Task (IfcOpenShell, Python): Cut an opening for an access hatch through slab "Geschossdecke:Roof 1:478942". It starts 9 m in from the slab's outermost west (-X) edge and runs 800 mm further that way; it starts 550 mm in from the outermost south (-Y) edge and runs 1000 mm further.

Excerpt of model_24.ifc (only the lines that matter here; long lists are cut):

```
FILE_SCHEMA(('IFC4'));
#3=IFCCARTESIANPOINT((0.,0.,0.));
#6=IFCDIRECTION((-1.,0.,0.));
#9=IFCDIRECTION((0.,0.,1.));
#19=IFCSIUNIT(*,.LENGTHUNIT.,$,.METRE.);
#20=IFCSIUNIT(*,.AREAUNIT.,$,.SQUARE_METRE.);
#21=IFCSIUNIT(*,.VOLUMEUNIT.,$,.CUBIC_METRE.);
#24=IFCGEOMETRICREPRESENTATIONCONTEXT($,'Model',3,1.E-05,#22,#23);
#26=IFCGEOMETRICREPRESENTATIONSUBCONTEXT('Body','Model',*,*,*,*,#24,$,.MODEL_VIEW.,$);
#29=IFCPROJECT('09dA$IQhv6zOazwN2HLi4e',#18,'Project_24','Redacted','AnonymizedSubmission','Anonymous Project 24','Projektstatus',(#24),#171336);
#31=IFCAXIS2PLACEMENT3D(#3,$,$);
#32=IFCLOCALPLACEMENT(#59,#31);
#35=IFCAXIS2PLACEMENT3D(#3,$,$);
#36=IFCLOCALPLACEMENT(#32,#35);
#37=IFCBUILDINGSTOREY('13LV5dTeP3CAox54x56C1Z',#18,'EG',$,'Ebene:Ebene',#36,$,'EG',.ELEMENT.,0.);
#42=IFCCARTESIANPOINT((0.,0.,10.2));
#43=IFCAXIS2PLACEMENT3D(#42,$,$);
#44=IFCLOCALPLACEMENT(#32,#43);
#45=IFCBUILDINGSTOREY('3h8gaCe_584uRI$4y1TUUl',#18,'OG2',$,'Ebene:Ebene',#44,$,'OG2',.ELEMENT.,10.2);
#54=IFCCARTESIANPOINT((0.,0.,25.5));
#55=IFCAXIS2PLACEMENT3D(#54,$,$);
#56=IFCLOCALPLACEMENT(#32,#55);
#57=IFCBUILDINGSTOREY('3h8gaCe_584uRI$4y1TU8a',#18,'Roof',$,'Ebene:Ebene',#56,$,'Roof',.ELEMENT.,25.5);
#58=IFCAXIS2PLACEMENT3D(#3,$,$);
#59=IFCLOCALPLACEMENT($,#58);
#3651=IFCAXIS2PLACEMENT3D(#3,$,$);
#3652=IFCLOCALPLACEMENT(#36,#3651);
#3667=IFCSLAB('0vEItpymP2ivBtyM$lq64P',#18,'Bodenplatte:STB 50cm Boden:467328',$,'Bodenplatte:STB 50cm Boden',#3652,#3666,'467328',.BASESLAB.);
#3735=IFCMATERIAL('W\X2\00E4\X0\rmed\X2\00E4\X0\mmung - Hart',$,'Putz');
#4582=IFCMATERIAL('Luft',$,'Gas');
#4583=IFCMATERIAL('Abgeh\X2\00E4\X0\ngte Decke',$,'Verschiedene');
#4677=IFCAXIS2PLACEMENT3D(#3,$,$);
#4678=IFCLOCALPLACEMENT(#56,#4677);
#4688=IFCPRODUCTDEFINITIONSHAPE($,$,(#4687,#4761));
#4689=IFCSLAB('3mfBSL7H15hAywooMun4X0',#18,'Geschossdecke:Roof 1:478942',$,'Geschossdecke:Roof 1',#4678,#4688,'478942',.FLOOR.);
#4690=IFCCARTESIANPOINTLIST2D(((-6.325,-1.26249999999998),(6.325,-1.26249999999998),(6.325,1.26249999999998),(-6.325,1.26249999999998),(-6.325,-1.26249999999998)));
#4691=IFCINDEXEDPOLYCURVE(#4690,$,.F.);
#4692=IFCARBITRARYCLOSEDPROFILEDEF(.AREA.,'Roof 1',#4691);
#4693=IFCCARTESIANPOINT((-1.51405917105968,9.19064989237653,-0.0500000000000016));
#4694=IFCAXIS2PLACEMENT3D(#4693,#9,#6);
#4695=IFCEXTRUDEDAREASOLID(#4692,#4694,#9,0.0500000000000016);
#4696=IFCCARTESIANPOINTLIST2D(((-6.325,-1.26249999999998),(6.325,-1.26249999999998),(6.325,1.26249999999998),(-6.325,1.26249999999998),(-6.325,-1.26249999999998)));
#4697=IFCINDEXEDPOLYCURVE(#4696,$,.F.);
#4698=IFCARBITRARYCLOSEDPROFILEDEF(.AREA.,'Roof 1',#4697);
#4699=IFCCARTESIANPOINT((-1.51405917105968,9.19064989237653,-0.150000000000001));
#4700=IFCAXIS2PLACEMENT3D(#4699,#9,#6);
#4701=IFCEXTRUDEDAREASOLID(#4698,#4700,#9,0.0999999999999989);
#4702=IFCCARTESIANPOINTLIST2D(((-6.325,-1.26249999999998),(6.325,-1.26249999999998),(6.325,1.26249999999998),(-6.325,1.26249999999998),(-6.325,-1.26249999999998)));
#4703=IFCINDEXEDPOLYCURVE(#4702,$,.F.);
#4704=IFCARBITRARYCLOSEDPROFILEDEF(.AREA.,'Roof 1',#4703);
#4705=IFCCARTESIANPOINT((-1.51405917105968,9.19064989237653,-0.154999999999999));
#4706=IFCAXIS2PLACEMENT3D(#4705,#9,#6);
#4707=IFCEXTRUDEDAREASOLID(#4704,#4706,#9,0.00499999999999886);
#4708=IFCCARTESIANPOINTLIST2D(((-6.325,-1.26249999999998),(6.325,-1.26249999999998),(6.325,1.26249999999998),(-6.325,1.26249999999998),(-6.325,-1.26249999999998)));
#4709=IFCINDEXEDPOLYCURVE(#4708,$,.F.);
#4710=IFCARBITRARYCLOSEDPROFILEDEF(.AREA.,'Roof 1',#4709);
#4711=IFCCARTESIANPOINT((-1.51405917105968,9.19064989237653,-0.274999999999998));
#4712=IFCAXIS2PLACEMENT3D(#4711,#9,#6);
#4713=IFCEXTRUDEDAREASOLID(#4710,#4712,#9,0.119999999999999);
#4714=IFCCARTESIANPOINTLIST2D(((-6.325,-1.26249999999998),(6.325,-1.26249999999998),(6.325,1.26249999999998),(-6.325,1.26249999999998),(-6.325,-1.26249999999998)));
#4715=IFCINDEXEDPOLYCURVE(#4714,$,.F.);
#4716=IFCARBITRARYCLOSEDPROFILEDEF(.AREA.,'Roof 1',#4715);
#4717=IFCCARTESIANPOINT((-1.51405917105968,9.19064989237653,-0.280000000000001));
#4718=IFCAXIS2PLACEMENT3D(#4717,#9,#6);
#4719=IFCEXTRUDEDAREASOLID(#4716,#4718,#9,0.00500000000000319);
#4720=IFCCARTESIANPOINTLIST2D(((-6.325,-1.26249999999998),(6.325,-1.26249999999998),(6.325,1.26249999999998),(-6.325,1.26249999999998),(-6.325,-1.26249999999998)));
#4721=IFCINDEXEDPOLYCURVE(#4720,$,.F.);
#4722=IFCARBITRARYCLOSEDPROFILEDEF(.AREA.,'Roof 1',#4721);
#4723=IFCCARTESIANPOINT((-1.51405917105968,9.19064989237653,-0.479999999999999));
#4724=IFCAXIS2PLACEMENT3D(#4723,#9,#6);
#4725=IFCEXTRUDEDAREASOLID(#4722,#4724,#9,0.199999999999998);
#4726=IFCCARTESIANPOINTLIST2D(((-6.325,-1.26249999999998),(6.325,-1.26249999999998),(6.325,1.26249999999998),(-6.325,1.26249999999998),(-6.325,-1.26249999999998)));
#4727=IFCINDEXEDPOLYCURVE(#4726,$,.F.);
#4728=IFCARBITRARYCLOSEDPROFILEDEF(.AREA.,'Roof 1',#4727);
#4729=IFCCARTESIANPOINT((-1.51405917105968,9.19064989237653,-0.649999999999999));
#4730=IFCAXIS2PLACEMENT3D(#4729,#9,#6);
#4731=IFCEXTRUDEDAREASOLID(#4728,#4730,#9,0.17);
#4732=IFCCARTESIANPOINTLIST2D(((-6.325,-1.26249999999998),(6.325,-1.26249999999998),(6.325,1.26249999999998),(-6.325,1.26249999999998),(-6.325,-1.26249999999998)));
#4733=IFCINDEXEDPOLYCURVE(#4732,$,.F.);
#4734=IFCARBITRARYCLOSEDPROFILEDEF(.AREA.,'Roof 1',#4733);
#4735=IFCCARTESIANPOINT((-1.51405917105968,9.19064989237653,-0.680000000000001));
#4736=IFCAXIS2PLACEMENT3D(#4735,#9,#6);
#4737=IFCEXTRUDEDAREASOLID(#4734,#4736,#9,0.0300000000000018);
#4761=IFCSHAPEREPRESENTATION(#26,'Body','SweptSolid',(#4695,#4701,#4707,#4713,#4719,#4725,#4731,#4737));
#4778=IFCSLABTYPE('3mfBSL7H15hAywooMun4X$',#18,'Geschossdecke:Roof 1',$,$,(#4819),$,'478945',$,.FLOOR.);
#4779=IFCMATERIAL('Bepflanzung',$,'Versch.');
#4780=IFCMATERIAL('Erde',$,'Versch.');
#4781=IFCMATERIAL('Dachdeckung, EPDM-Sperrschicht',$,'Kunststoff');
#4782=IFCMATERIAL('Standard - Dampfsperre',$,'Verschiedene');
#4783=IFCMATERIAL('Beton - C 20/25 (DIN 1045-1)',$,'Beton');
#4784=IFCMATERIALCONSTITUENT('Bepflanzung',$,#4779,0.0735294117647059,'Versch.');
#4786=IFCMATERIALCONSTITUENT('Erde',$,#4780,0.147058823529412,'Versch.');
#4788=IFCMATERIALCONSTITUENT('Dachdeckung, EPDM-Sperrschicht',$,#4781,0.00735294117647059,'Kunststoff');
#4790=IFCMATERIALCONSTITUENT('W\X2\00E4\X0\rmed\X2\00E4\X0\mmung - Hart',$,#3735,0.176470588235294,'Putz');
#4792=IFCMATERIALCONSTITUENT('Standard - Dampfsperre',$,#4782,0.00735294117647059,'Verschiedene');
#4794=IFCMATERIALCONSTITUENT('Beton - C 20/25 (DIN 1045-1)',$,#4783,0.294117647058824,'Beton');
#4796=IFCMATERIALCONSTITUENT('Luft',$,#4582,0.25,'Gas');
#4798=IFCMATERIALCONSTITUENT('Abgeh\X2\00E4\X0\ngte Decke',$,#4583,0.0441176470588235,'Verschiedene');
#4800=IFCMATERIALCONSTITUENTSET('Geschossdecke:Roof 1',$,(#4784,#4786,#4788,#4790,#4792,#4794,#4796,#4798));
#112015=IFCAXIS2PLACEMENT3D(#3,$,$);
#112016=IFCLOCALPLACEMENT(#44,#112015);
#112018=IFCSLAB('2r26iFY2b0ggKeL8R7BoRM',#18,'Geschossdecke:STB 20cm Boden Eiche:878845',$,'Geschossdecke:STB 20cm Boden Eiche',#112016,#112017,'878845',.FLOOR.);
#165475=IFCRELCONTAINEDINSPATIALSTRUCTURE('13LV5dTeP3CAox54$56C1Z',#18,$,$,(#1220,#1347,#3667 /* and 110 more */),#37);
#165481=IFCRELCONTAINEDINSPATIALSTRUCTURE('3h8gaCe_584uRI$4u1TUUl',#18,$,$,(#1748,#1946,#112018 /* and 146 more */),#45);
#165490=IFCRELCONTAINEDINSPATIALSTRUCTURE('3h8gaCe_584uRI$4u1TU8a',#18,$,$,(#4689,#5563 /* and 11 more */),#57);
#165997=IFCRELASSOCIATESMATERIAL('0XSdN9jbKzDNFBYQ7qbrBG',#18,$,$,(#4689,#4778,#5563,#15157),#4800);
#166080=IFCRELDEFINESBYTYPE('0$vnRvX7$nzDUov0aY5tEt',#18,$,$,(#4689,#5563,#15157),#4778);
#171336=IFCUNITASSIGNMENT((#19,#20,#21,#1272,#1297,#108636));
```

```python
import numpy as np
import ifcopenshell
import ifcopenshell.api.feature
import ifcopenshell.api.geometry
import ifcopenshell.api.root
import ifcopenshell.geom
import ifcopenshell.util.placement
import ifcopenshell.util.representation
import ifcopenshell.util.shape
import ifcopenshell.util.unit

model = ifcopenshell.open("model_24.ifc")
unit_scale = ifcopenshell.util.unit.calculate_unit_scale(model)
settings = ifcopenshell.geom.settings()


def volume(element):
    """Net volume in cubic metres, openings subtracted."""
    shape = ifcopenshell.geom.create_shape(settings, element)
    return ifcopenshell.util.shape.get_volume(shape.geometry)


slab = model.by_guid("3mfBSL7H15hAywooMun4X0")
before = volume(slab)

# Extent in the slab's own axes, in metres. The edges named are its -X and -Y sides.
slab_shape = ifcopenshell.geom.create_shape(settings, slab)
vertices = ifcopenshell.util.shape.get_vertices(slab_shape.geometry)
x_min, y_min, bottom = vertices.min(axis=0)
top = vertices[:, 2].max()

opening = ifcopenshell.api.root.create_entity(model, ifc_class="IfcOpeningElement", name="Access hatch opening", predefined_type="OPENING")
context = ifcopenshell.util.representation.get_context(model, "Model", "Body", "MODEL_VIEW")
width, depth = 0.8, 1
outline = [(0.0, 0.0), (width, 0.0), (width, depth), (0.0, depth), (0.0, 0.0)]
# Overshoot both faces by 50 mm so the cut is clean.
shape = ifcopenshell.api.geometry.add_slab_representation(
    model, context=context, depth=top - bottom + 0.1, polyline=outline
)
ifcopenshell.api.geometry.assign_representation(model, product=opening, representation=shape)

matrix = ifcopenshell.util.placement.get_local_placement(slab.ObjectPlacement)
matrix[:, 3] = matrix @ np.append(np.array([x_min + 9, y_min + 0.55, bottom - 0.05]) / unit_scale, 1.0)
ifcopenshell.api.geometry.edit_object_placement(model, product=opening, matrix=matrix, is_si=False)
ifcopenshell.api.feature.add_feature(model, feature=opening, element=slab)

after = volume(slab)

print(f"slab volume {before:.3f} -> {after:.3f} m3")

model.write("model_24_rev.ifc")
```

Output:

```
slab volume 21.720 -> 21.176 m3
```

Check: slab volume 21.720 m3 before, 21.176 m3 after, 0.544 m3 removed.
